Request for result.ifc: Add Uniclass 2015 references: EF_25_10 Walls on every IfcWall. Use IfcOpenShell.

First a look at what the model holds.

```python
import ifcopenshell

model = ifcopenshell.open("result.ifc")
print(model.schema)
print("classifications:", [c.Name for c in model.by_type("IfcClassification")])
for ifc_class in ("IfcDoor", "IfcRoof", "IfcStair", "IfcWall", "IfcWindow"):
    print(ifc_class, len(model.by_type(ifc_class)))
```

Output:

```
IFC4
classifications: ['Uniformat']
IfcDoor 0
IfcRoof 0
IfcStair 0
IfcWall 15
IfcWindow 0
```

```python
import ifcopenshell
import ifcopenshell.api.classification

model = ifcopenshell.open("result.ifc")

system = ifcopenshell.api.classification.add_classification(model, classification="Uniclass 2015")

codes = {
    "IfcWall": ("EF_25_10", "Walls"),
}
for ifc_class, (code, name) in codes.items():
    products = model.by_type(ifc_class)
    ifcopenshell.api.classification.add_reference(
        model, products=products, classification=system, identification=code, name=name
    )
    print(code, len(products))

model.write("result_edited.ifc")
```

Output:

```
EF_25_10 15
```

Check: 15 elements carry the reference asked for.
